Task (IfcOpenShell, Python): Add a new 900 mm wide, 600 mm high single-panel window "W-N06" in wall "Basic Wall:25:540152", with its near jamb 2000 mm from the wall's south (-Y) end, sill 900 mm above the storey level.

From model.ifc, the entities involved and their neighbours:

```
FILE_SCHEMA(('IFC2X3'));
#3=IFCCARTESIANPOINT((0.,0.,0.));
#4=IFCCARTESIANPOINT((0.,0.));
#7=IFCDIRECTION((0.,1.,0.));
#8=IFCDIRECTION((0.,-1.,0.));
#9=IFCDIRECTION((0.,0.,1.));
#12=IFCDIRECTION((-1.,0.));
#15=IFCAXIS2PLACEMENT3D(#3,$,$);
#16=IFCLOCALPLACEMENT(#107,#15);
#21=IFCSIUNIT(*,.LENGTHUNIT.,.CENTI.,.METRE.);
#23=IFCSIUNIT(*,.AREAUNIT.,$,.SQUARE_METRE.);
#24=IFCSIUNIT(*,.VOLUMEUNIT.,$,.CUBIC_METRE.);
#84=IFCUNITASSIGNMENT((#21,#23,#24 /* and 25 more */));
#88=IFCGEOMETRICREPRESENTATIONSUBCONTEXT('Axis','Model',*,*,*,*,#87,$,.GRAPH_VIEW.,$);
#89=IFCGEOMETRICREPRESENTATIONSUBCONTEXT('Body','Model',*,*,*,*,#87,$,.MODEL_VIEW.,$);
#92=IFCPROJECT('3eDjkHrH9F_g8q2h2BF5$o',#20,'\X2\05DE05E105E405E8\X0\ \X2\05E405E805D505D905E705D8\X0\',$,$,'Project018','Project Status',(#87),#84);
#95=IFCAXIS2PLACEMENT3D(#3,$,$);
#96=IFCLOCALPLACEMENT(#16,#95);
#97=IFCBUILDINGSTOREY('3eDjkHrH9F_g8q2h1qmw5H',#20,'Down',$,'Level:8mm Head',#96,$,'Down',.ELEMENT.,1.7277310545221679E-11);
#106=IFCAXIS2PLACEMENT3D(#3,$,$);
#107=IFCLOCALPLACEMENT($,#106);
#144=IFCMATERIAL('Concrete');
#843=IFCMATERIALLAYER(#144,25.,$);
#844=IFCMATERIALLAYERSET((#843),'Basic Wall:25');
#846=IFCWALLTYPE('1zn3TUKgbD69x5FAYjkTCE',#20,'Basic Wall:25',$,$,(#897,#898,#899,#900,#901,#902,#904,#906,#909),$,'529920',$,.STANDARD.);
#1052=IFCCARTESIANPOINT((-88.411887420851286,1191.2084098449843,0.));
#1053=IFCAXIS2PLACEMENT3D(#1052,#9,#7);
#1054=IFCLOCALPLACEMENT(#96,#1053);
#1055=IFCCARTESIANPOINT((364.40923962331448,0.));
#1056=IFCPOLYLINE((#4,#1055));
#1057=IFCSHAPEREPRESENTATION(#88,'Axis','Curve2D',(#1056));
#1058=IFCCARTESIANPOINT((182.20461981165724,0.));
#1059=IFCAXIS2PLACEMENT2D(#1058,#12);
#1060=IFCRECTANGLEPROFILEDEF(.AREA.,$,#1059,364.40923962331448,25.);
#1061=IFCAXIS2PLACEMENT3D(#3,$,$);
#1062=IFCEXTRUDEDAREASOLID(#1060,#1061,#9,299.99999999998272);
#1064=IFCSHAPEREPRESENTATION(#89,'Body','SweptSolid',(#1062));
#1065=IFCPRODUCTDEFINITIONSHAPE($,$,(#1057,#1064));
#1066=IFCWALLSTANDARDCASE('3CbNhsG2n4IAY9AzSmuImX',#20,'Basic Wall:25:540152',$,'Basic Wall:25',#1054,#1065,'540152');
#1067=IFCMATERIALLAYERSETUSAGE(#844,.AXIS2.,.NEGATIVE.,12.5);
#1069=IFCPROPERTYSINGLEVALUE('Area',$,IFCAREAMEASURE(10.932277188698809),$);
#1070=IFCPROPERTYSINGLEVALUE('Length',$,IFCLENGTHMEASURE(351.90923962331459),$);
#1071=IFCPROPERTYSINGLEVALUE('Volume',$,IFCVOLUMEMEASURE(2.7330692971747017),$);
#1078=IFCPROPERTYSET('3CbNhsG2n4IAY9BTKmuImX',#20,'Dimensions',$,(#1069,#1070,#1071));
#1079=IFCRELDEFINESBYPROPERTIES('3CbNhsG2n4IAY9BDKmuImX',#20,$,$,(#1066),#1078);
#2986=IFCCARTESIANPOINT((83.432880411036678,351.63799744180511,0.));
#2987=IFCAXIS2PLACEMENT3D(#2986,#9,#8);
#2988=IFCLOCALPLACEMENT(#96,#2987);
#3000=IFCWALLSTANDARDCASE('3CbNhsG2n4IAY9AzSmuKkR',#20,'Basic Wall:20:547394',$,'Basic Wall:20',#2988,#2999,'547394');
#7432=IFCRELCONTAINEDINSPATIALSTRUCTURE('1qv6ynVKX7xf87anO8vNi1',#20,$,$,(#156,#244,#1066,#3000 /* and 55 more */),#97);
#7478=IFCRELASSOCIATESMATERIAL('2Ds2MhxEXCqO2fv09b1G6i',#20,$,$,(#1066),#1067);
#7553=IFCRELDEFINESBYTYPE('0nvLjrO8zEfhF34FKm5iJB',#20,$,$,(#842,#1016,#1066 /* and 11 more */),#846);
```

```python
import numpy as np
import ifcopenshell
import ifcopenshell.api.feature
import ifcopenshell.api.geometry
import ifcopenshell.api.pset
import ifcopenshell.api.root
import ifcopenshell.api.spatial
import ifcopenshell.api.type
import ifcopenshell.geom
import ifcopenshell.util.element
import ifcopenshell.util.placement
import ifcopenshell.util.representation
import ifcopenshell.util.shape
import ifcopenshell.util.unit

model = ifcopenshell.open("model.ifc")
unit_scale = ifcopenshell.util.unit.calculate_unit_scale(model)
area_scale = ifcopenshell.util.unit.calculate_unit_scale(model, "AREAUNIT")
volume_scale = ifcopenshell.util.unit.calculate_unit_scale(model, "VOLUMEUNIT")
settings = ifcopenshell.geom.settings()


def volume(element):
    """Net volume in cubic metres, openings subtracted."""
    shape = ifcopenshell.geom.create_shape(settings, element)
    return ifcopenshell.util.shape.get_volume(shape.geometry)


wall = model.by_guid("3CbNhsG2n4IAY9AzSmuImX")
storey = ifcopenshell.util.element.get_container(wall, ifc_class="IfcBuildingStorey")
context = ifcopenshell.util.representation.get_context(model, "Model", "Body", "MODEL_VIEW")
before = volume(wall)

width, height, from_end, sill = 0.9, 0.6, 2, 0.9  # metres

# The wall runs along its own X axis, and the end named is its -X end.
wall_shape = ifcopenshell.geom.create_shape(settings, wall)
x, y, z = ifcopenshell.util.shape.get_vertices(wall_shape.geometry).T
start = x.min() + from_end
face, thickness = float(y.min()), float(y.max() - y.min())
wall_matrix = ifcopenshell.util.placement.get_local_placement(wall.ObjectPlacement)
level = ifcopenshell.util.placement.get_local_placement(storey.ObjectPlacement)[2, 3]


def in_wall(x, y):
    """Placement at x, y metres in the wall's axes, at sill height."""
    matrix = wall_matrix.copy()
    matrix[:, 3] = wall_matrix @ np.array([x / unit_scale, y / unit_scale, 0.0, 1.0])
    matrix[2, 3] = level + sill / unit_scale
    return matrix


# Opening: a box that overshoots both wall faces by 50 mm.
opening = ifcopenshell.api.root.create_entity(model, ifc_class="IfcOpeningElement")
box = ifcopenshell.api.geometry.add_wall_representation(
    model, context=context, length=width, height=height, thickness=thickness + 0.1
)
ifcopenshell.api.geometry.assign_representation(model, product=opening, representation=box)
ifcopenshell.api.geometry.edit_object_placement(model, product=opening, matrix=in_wall(start, face - 0.05), is_si=False)
ifcopenshell.api.feature.add_feature(model, feature=opening, element=wall)

window = ifcopenshell.api.root.create_entity(model, ifc_class="IfcWindow", name="W-N06")
window.OverallWidth, window.OverallHeight = width / unit_scale, height / unit_scale
body = ifcopenshell.api.geometry.add_window_representation(
    model,
    context=context,
    overall_width=window.OverallWidth,
    overall_height=window.OverallHeight,
    partition_type="SINGLE_PANEL",
)
ifcopenshell.api.geometry.assign_representation(model, product=window, representation=body)
ifcopenshell.api.spatial.assign_container(model, products=[window], relating_structure=storey)
fills = ifcopenshell.api.feature.add_filling(model, opening=opening, element=window)
fills.OwnerHistory = window.OwnerHistory  # required in IFC2X3

# IFC2X3 keeps the operation on the window style.
style = ifcopenshell.api.root.create_entity(model, ifc_class="IfcWindowStyle", name="W-N06")
style.OperationType, style.ConstructionType = "SINGLE_PANEL", "NOTDEFINED"
style.ParameterTakesPrecedence = style.Sizeable = False
ifcopenshell.api.type.assign_type(model, related_objects=[window], relating_type=style)

# Centre the window in the wall's thickness.
ifcopenshell.api.geometry.edit_object_placement(model, product=window, matrix=in_wall(start, face), is_si=False)
window_shape = ifcopenshell.geom.create_shape(settings, window)
depth = ifcopenshell.util.shape.get_vertices(window_shape.geometry)[:, 1]
offset = face + thickness / 2 - (depth.min() + depth.max()) / 2
ifcopenshell.api.geometry.edit_object_placement(model, product=window, matrix=in_wall(start, offset), is_si=False)

after = volume(wall)

# Update the wall's stored quantities.
pset = model.by_id(ifcopenshell.util.element.get_pset(wall, "Dimensions", should_inherit=False)["id"])
ifcopenshell.api.pset.edit_pset(model, pset=pset, properties={
    "Area": model.create_entity("IfcAreaMeasure", after / thickness / area_scale),
    "Volume": model.create_entity("IfcVolumeMeasure", after / volume_scale),
})

print(f"wall volume {before:.3f} -> {after:.3f} m3")

model.write("model_updated.ifc")
```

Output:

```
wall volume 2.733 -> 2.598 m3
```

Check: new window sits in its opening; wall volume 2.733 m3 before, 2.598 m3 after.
